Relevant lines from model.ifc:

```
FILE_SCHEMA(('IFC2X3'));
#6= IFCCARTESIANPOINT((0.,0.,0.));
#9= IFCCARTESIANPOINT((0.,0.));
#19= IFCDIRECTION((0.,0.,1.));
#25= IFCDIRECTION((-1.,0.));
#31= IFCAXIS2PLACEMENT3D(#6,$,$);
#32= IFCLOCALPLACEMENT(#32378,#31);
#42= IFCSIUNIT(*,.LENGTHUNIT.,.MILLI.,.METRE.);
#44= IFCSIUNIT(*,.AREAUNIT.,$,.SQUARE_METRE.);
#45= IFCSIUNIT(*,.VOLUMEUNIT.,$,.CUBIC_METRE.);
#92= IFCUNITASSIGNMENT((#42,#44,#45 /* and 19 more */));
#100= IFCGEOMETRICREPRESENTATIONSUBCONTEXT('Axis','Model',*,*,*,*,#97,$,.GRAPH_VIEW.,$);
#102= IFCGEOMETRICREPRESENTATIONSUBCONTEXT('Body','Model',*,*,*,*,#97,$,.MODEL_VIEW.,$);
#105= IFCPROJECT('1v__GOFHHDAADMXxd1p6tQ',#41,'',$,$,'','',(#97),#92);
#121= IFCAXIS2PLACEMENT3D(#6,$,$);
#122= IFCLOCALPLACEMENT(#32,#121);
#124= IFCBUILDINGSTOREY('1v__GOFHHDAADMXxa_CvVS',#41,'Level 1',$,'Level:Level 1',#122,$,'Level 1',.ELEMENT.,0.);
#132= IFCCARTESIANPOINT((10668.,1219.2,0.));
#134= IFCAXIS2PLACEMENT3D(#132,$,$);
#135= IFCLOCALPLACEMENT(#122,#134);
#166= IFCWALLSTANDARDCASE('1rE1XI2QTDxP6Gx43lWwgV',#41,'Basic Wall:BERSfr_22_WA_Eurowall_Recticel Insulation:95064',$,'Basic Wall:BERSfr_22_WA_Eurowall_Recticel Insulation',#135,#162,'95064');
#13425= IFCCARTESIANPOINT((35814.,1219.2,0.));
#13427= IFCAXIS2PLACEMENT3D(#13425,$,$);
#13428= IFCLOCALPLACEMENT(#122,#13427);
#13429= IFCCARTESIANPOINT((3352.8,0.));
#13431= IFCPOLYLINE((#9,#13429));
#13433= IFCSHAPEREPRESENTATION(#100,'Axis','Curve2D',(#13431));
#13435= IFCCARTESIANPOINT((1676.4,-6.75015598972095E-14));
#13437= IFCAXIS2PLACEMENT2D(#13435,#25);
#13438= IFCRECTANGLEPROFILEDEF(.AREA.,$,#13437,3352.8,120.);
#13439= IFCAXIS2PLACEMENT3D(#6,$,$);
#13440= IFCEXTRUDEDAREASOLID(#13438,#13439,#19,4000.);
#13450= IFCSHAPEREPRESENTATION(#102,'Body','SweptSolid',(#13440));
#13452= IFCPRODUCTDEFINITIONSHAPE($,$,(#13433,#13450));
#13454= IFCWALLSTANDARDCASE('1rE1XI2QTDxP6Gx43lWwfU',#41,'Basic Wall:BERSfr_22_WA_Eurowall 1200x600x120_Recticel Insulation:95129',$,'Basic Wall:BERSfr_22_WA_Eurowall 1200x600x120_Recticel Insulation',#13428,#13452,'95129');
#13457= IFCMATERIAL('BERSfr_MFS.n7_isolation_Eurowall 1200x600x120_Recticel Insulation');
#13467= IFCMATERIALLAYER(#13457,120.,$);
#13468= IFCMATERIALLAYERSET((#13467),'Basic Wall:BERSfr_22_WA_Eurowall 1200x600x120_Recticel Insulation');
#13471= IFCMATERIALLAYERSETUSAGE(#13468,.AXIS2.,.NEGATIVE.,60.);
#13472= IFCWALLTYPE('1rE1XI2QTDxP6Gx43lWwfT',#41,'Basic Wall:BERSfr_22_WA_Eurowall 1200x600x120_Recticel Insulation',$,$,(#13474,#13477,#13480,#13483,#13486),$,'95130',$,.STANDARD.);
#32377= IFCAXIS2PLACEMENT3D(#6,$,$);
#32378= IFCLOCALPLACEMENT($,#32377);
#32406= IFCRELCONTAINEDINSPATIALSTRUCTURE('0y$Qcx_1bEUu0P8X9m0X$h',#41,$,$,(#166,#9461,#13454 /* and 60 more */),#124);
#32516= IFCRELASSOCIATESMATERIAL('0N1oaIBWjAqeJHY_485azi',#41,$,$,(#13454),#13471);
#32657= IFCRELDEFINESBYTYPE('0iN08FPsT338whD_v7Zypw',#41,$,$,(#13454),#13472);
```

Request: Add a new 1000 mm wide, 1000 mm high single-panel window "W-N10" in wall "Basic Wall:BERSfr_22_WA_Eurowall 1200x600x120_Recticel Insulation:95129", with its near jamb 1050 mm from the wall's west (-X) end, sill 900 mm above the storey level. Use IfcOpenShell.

```python
import numpy as np
import ifcopenshell
import ifcopenshell.api.feature
import ifcopenshell.api.geometry
import ifcopenshell.api.root
import ifcopenshell.api.spatial
import ifcopenshell.api.type
import ifcopenshell.geom
import ifcopenshell.util.element
import ifcopenshell.util.placement
import ifcopenshell.util.representation
import ifcopenshell.util.shape
import ifcopenshell.util.unit

model = ifcopenshell.open("model.ifc")
unit_scale = ifcopenshell.util.unit.calculate_unit_scale(model)
settings = ifcopenshell.geom.settings()


def volume(element):
    """Net volume in cubic metres, openings subtracted."""
    shape = ifcopenshell.geom.create_shape(settings, element)
    return ifcopenshell.util.shape.get_volume(shape.geometry)


wall = model.by_guid("1rE1XI2QTDxP6Gx43lWwfU")
storey = ifcopenshell.util.element.get_container(wall, ifc_class="IfcBuildingStorey")
context = ifcopenshell.util.representation.get_context(model, "Model", "Body", "MODEL_VIEW")
before = volume(wall)

width, height, from_end, sill = 1, 1, 1.05, 0.9  # metres

# The wall runs along its own X axis, and the end named is its -X end.
wall_shape = ifcopenshell.geom.create_shape(settings, wall)
x, y, z = ifcopenshell.util.shape.get_vertices(wall_shape.geometry).T
start = x.min() + from_end
face, thickness = float(y.min()), float(y.max() - y.min())
wall_matrix = ifcopenshell.util.placement.get_local_placement(wall.ObjectPlacement)
level = ifcopenshell.util.placement.get_local_placement(storey.ObjectPlacement)[2, 3]


def in_wall(x, y):
    """Placement at x, y metres in the wall's axes, at sill height."""
    matrix = wall_matrix.copy()
    matrix[:, 3] = wall_matrix @ np.array([x / unit_scale, y / unit_scale, 0.0, 1.0])
    matrix[2, 3] = level + sill / unit_scale
    return matrix


# Opening: a box that overshoots both wall faces by 50 mm.
opening = ifcopenshell.api.root.create_entity(model, ifc_class="IfcOpeningElement")
box = ifcopenshell.api.geometry.add_wall_representation(
    model, context=context, length=width, height=height, thickness=thickness + 0.1
)
ifcopenshell.api.geometry.assign_representation(model, product=opening, representation=box)
ifcopenshell.api.geometry.edit_object_placement(model, product=opening, matrix=in_wall(start, face - 0.05), is_si=False)
ifcopenshell.api.feature.add_feature(model, feature=opening, element=wall)

window = ifcopenshell.api.root.create_entity(model, ifc_class="IfcWindow", name="W-N10")
window.OverallWidth, window.OverallHeight = width / unit_scale, height / unit_scale
body = ifcopenshell.api.geometry.add_window_representation(
    model,
    context=context,
    overall_width=window.OverallWidth,
    overall_height=window.OverallHeight,
    partition_type="SINGLE_PANEL",
)
ifcopenshell.api.geometry.assign_representation(model, product=window, representation=body)
ifcopenshell.api.spatial.assign_container(model, products=[window], relating_structure=storey)
fills = ifcopenshell.api.feature.add_filling(model, opening=opening, element=window)
fills.OwnerHistory = window.OwnerHistory  # required in IFC2X3

# IFC2X3 keeps the operation on the window style.
style = ifcopenshell.api.root.create_entity(model, ifc_class="IfcWindowStyle", name="W-N10")
style.OperationType, style.ConstructionType = "SINGLE_PANEL", "NOTDEFINED"
style.ParameterTakesPrecedence = style.Sizeable = False
ifcopenshell.api.type.assign_type(model, related_objects=[window], relating_type=style)

# Centre the window in the wall's thickness.
ifcopenshell.api.geometry.edit_object_placement(model, product=window, matrix=in_wall(start, face), is_si=False)
window_shape = ifcopenshell.geom.create_shape(settings, window)
depth = ifcopenshell.util.shape.get_vertices(window_shape.geometry)[:, 1]
offset = face + thickness / 2 - (depth.min() + depth.max()) / 2
ifcopenshell.api.geometry.edit_object_placement(model, product=window, matrix=in_wall(start, offset), is_si=False)

after = volume(wall)

print(f"wall volume {before:.3f} -> {after:.3f} m3")

model.write("model_edited.ifc")
```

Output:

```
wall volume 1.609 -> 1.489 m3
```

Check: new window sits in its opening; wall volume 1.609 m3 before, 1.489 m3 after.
